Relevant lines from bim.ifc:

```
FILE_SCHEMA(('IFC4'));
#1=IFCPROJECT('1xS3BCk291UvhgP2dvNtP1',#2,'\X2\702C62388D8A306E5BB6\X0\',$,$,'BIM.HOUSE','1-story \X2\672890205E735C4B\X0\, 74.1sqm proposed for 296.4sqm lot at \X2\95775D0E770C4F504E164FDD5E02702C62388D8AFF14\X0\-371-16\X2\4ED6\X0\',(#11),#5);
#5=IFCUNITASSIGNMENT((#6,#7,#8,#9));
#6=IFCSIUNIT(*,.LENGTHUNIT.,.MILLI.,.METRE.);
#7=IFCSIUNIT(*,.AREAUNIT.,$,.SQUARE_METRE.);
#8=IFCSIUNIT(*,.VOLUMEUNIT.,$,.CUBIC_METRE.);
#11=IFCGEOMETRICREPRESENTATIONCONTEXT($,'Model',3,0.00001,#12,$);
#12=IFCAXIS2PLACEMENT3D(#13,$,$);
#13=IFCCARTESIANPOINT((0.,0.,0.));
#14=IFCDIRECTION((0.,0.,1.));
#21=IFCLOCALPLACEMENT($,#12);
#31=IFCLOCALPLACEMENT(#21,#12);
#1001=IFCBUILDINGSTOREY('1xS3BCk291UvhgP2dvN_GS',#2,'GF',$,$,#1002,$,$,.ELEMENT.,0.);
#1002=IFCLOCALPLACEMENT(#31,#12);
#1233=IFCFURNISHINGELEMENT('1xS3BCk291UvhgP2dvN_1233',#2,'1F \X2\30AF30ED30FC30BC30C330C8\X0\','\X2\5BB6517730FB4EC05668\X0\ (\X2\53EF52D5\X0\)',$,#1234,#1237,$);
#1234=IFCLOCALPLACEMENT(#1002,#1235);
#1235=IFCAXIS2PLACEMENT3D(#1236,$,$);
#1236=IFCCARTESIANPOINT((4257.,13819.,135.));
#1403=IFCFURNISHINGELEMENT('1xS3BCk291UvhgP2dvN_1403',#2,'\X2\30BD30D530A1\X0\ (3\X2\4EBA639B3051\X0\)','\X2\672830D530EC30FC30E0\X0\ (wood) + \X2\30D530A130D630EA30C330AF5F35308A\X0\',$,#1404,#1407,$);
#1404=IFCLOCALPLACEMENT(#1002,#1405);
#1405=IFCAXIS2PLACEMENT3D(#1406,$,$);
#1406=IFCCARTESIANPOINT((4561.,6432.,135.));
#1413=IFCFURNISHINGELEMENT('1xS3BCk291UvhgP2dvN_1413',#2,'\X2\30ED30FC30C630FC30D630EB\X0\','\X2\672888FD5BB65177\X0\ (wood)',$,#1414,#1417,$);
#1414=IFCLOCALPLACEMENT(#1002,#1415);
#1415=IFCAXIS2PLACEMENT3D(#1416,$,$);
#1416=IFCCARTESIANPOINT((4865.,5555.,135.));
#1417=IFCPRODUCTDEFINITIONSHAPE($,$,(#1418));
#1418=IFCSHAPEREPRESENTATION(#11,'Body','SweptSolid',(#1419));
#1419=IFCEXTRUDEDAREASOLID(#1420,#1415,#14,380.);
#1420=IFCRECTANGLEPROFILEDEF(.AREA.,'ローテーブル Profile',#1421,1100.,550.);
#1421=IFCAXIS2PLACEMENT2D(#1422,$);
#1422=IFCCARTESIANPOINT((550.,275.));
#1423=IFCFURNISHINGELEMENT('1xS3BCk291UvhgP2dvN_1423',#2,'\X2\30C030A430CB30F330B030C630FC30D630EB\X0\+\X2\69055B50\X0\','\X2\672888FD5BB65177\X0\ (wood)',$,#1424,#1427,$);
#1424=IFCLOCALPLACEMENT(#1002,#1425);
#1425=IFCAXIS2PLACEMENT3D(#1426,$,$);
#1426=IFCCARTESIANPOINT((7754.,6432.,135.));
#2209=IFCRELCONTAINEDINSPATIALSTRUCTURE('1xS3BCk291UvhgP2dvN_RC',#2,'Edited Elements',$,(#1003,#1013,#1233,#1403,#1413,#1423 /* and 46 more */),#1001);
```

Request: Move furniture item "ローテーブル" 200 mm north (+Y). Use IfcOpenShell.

```python
import ifcopenshell
import ifcopenshell.api.geometry
import ifcopenshell.util.placement
import ifcopenshell.util.unit

model = ifcopenshell.open("bim.ifc")
unit_scale = ifcopenshell.util.unit.calculate_unit_scale(model)

item = model.by_guid("1xS3BCk291UvhgP2dvN_1413")
matrix = ifcopenshell.util.placement.get_local_placement(item.ObjectPlacement)
matrix[1, 3] += 0.2 / unit_scale
ifcopenshell.api.geometry.edit_object_placement(model, product=item, matrix=matrix, is_si=False)

print(ifcopenshell.util.placement.get_local_placement(item.ObjectPlacement).round(3) + 0.0)

model.write("bim_edited.ifc")
```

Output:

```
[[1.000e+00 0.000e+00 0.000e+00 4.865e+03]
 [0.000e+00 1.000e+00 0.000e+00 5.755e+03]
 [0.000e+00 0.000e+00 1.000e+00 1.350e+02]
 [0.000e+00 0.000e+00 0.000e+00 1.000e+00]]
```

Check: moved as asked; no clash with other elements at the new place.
